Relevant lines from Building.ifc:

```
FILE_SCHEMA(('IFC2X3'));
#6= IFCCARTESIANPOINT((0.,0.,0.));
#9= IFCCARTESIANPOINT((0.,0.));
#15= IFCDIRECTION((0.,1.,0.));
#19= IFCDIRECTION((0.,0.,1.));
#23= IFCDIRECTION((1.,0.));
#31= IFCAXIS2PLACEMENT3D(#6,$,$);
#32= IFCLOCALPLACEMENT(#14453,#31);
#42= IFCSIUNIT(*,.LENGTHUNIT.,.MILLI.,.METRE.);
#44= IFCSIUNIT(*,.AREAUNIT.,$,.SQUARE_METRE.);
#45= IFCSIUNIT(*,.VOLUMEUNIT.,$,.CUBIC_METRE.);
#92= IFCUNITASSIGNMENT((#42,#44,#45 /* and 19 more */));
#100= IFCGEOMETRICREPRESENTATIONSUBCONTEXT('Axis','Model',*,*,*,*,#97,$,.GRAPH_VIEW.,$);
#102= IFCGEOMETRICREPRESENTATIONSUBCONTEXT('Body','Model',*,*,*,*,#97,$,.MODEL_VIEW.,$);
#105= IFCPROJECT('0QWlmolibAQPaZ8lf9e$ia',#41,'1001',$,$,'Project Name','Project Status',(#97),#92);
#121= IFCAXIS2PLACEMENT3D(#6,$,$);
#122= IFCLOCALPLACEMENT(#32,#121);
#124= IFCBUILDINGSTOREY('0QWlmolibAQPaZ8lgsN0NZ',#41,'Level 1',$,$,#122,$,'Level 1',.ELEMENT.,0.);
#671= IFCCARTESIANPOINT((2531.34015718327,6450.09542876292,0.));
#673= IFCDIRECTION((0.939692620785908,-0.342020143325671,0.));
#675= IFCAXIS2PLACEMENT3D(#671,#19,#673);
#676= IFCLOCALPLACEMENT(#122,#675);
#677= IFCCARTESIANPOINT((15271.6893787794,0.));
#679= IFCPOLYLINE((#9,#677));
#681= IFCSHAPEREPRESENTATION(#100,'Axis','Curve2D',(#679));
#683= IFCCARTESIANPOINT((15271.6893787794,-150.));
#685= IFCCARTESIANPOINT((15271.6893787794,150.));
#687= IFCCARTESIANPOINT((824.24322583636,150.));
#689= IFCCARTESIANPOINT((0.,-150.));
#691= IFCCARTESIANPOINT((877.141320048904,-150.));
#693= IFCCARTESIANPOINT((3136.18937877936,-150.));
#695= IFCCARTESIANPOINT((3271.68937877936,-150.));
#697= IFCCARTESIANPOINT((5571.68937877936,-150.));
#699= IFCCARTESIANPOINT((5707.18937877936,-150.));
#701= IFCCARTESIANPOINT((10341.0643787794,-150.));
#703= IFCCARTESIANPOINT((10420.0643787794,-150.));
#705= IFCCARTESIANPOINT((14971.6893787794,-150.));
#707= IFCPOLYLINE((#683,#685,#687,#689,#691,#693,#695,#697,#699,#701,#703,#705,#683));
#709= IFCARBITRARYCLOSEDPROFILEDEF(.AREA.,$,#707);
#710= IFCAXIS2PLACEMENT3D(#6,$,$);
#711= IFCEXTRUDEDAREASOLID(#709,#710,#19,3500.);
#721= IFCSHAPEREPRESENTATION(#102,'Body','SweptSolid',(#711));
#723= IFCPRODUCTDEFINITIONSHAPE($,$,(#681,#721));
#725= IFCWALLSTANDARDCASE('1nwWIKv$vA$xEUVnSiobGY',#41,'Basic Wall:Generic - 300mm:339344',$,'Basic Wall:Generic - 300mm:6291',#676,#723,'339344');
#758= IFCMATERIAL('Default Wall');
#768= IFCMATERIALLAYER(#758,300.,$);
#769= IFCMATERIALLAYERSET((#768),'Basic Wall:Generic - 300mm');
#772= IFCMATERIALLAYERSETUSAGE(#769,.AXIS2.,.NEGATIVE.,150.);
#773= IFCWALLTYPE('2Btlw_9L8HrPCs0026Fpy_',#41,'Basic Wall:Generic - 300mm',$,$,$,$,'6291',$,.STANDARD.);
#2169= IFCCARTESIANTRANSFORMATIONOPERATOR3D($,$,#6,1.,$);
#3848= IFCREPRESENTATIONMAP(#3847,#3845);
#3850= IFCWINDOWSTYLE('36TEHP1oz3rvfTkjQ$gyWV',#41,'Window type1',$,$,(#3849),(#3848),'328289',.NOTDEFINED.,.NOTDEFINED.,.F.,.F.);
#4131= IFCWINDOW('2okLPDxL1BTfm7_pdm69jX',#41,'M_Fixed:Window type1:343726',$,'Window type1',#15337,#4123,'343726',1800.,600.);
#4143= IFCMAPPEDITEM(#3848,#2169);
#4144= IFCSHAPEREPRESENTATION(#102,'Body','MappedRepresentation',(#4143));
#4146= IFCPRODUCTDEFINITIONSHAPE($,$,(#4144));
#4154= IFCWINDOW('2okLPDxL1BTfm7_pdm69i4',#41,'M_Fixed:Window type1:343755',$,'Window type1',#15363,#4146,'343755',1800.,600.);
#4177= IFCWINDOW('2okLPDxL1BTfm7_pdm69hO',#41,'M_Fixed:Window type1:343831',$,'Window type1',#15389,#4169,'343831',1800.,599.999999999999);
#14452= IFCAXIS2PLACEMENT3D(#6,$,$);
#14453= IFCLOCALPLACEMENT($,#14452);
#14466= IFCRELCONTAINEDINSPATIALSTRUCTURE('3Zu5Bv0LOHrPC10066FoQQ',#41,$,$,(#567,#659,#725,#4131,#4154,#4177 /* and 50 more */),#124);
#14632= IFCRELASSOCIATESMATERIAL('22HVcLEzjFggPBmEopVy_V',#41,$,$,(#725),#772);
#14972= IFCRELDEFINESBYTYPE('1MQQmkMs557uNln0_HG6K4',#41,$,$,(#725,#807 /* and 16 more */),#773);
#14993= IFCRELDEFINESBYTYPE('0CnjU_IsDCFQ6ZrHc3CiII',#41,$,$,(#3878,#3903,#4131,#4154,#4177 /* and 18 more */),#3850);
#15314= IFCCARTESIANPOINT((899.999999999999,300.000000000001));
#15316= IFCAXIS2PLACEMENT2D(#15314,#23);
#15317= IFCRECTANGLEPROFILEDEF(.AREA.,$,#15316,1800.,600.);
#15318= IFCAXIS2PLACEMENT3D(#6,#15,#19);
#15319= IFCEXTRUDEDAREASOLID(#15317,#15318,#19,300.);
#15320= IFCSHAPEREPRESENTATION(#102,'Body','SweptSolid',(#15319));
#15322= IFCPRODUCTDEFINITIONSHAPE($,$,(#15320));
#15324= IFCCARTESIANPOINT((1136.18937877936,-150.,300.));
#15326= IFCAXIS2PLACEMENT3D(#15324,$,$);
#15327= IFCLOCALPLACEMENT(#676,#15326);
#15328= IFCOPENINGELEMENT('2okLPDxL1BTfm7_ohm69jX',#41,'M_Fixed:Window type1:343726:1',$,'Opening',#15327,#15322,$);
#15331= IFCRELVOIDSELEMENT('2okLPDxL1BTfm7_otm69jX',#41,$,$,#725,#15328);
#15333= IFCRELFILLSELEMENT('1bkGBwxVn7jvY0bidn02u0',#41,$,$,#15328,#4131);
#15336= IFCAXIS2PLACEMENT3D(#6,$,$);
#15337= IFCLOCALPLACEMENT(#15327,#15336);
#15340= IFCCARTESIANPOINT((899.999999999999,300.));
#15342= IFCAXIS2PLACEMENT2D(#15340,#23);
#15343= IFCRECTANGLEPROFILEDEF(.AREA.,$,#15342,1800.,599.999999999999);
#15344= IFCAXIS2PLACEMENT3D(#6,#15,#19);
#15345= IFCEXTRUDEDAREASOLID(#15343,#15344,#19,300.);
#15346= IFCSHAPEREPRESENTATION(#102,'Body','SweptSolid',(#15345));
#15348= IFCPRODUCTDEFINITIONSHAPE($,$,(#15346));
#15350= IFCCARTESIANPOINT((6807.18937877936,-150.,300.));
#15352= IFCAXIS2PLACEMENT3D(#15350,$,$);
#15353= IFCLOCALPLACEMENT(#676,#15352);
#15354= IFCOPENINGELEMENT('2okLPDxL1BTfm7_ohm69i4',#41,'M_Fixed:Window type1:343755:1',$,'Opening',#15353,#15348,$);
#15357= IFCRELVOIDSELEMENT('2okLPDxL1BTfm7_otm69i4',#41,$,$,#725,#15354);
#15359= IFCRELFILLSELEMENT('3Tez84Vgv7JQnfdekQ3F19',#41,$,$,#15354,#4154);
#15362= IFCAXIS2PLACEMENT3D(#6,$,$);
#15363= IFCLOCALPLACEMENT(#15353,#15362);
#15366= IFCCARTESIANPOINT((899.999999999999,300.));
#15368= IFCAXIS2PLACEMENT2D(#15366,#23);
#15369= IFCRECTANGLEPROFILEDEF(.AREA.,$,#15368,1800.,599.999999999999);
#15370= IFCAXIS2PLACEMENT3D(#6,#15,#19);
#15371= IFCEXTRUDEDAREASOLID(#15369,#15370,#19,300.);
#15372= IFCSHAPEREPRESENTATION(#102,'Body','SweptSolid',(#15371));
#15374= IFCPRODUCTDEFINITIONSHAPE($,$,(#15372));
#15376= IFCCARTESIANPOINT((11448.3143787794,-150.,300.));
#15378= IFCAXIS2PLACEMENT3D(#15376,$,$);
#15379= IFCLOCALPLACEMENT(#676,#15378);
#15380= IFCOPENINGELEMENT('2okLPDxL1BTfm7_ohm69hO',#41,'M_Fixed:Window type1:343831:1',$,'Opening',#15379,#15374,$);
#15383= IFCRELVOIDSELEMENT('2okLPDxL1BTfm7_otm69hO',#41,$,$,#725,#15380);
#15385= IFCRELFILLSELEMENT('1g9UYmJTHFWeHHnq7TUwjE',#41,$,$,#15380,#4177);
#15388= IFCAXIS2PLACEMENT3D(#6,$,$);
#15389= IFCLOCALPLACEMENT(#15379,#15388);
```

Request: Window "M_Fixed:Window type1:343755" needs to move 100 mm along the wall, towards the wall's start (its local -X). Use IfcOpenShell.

```python
import ifcopenshell
import ifcopenshell.api.geometry
import ifcopenshell.util.placement
import ifcopenshell.util.unit

model = ifcopenshell.open("Building.ifc")
unit_scale = ifcopenshell.util.unit.calculate_unit_scale(model)

window = model.by_guid("2okLPDxL1BTfm7_pdm69i4")
opening = window.FillsVoids[0].RelatingOpeningElement
wall = opening.VoidsElements[0].RelatingBuildingElement

wall_matrix = ifcopenshell.util.placement.get_local_placement(wall.ObjectPlacement)
shift = wall_matrix[:3, 0] * -0.1 / unit_scale
before = ifcopenshell.util.placement.get_local_placement(window.ObjectPlacement)[:3, 3].copy()

# The window is placed relative to its opening, so it follows when the opening moves.
matrix = ifcopenshell.util.placement.get_local_placement(opening.ObjectPlacement)
matrix[:3, 3] += shift
ifcopenshell.api.geometry.edit_object_placement(
    model, product=opening, matrix=matrix, is_si=False, should_transform_children=True
)

after = ifcopenshell.util.placement.get_local_placement(window.ObjectPlacement)[:3, 3]
print("window moved by", (after - before).round(3) + 0.0)

model.write("Building_rev.ifc")
```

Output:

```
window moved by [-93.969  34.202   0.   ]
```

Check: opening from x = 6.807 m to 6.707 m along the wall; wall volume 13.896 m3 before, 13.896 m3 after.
